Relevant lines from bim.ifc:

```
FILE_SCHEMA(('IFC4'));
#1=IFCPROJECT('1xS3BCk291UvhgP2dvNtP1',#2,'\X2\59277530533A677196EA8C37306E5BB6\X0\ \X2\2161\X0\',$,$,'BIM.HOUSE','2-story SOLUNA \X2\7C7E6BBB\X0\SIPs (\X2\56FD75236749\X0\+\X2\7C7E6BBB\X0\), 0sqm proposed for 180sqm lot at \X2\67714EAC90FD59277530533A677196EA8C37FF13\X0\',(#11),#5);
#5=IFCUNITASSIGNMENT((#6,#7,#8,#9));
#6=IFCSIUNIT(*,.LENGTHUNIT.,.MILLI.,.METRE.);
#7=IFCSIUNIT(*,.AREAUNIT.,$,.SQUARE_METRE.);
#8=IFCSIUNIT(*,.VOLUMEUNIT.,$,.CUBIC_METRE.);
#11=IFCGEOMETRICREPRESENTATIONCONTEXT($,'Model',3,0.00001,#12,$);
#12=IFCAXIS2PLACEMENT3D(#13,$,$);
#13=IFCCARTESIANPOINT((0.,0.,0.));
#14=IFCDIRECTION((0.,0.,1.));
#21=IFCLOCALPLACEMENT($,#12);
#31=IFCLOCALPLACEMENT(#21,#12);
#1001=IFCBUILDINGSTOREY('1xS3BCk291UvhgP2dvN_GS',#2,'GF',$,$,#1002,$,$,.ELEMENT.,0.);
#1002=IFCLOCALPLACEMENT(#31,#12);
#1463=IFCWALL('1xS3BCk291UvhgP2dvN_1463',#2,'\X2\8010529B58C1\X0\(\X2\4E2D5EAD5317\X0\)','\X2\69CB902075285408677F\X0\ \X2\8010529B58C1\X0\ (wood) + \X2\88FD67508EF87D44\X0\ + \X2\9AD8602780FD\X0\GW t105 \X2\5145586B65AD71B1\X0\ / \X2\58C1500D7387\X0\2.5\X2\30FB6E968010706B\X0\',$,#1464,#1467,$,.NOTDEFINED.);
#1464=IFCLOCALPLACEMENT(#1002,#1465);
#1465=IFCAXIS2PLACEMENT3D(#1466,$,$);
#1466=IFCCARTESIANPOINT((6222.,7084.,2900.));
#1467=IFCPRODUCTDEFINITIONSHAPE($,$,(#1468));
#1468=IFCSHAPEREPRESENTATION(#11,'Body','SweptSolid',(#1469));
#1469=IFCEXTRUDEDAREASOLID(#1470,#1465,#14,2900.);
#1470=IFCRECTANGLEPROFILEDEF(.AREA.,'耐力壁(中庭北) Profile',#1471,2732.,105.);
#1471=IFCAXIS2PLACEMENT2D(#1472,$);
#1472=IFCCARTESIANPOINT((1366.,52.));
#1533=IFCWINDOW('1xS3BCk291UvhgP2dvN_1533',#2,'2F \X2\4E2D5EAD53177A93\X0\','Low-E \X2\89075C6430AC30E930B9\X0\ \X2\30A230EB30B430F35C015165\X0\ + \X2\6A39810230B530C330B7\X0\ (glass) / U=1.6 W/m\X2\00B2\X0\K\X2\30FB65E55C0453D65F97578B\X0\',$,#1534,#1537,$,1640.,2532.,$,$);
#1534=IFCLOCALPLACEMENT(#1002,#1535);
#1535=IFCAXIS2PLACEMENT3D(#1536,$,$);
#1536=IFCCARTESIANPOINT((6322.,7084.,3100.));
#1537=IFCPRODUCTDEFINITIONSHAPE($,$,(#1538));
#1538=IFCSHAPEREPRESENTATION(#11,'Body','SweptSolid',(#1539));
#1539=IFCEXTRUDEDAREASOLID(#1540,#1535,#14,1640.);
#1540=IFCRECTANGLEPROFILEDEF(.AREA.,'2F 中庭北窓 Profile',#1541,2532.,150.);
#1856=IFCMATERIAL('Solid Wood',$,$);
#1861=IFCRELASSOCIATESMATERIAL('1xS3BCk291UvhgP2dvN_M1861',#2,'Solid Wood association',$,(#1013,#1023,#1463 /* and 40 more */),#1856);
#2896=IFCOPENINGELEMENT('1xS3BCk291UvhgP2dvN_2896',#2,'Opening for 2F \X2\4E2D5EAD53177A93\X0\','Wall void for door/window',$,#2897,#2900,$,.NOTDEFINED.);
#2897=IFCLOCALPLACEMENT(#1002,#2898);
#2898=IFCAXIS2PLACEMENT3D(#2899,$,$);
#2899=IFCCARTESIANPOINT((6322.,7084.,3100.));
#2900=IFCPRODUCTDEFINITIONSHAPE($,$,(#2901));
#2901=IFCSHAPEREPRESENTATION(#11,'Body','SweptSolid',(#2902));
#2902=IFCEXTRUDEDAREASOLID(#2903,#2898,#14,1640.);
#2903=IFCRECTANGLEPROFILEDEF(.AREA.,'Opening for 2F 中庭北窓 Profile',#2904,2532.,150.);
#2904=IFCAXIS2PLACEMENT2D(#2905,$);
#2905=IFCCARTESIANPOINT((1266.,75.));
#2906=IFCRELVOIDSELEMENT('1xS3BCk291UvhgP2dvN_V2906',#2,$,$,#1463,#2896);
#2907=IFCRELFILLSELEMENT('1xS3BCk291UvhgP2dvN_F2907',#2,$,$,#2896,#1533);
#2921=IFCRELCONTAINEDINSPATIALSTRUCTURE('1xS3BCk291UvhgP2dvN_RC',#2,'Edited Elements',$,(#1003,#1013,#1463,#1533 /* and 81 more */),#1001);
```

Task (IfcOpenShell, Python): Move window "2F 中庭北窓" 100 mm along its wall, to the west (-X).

```python
import ifcopenshell
import ifcopenshell.api.geometry
import ifcopenshell.util.placement
import ifcopenshell.util.unit

model = ifcopenshell.open("bim.ifc")
unit_scale = ifcopenshell.util.unit.calculate_unit_scale(model)

window = model.by_id(1533)
opening = window.FillsVoids[0].RelatingOpeningElement
wall = opening.VoidsElements[0].RelatingBuildingElement

wall_matrix = ifcopenshell.util.placement.get_local_placement(wall.ObjectPlacement)
shift = wall_matrix[:3, 0] * -0.1 / unit_scale
before = ifcopenshell.util.placement.get_local_placement(window.ObjectPlacement)[:3, 3].copy()

# The window is not placed relative to its opening, so move both.
for product in (opening, window):
    matrix = ifcopenshell.util.placement.get_local_placement(product.ObjectPlacement)
    matrix[:3, 3] += shift
    ifcopenshell.api.geometry.edit_object_placement(model, product=product, matrix=matrix, is_si=False)

after = ifcopenshell.util.placement.get_local_placement(window.ObjectPlacement)[:3, 3]
print("window moved by", (after - before).round(3) + 0.0)

model.write("bim_v2.ifc")
```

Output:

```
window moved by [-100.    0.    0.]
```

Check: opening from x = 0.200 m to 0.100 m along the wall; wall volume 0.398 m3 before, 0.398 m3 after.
